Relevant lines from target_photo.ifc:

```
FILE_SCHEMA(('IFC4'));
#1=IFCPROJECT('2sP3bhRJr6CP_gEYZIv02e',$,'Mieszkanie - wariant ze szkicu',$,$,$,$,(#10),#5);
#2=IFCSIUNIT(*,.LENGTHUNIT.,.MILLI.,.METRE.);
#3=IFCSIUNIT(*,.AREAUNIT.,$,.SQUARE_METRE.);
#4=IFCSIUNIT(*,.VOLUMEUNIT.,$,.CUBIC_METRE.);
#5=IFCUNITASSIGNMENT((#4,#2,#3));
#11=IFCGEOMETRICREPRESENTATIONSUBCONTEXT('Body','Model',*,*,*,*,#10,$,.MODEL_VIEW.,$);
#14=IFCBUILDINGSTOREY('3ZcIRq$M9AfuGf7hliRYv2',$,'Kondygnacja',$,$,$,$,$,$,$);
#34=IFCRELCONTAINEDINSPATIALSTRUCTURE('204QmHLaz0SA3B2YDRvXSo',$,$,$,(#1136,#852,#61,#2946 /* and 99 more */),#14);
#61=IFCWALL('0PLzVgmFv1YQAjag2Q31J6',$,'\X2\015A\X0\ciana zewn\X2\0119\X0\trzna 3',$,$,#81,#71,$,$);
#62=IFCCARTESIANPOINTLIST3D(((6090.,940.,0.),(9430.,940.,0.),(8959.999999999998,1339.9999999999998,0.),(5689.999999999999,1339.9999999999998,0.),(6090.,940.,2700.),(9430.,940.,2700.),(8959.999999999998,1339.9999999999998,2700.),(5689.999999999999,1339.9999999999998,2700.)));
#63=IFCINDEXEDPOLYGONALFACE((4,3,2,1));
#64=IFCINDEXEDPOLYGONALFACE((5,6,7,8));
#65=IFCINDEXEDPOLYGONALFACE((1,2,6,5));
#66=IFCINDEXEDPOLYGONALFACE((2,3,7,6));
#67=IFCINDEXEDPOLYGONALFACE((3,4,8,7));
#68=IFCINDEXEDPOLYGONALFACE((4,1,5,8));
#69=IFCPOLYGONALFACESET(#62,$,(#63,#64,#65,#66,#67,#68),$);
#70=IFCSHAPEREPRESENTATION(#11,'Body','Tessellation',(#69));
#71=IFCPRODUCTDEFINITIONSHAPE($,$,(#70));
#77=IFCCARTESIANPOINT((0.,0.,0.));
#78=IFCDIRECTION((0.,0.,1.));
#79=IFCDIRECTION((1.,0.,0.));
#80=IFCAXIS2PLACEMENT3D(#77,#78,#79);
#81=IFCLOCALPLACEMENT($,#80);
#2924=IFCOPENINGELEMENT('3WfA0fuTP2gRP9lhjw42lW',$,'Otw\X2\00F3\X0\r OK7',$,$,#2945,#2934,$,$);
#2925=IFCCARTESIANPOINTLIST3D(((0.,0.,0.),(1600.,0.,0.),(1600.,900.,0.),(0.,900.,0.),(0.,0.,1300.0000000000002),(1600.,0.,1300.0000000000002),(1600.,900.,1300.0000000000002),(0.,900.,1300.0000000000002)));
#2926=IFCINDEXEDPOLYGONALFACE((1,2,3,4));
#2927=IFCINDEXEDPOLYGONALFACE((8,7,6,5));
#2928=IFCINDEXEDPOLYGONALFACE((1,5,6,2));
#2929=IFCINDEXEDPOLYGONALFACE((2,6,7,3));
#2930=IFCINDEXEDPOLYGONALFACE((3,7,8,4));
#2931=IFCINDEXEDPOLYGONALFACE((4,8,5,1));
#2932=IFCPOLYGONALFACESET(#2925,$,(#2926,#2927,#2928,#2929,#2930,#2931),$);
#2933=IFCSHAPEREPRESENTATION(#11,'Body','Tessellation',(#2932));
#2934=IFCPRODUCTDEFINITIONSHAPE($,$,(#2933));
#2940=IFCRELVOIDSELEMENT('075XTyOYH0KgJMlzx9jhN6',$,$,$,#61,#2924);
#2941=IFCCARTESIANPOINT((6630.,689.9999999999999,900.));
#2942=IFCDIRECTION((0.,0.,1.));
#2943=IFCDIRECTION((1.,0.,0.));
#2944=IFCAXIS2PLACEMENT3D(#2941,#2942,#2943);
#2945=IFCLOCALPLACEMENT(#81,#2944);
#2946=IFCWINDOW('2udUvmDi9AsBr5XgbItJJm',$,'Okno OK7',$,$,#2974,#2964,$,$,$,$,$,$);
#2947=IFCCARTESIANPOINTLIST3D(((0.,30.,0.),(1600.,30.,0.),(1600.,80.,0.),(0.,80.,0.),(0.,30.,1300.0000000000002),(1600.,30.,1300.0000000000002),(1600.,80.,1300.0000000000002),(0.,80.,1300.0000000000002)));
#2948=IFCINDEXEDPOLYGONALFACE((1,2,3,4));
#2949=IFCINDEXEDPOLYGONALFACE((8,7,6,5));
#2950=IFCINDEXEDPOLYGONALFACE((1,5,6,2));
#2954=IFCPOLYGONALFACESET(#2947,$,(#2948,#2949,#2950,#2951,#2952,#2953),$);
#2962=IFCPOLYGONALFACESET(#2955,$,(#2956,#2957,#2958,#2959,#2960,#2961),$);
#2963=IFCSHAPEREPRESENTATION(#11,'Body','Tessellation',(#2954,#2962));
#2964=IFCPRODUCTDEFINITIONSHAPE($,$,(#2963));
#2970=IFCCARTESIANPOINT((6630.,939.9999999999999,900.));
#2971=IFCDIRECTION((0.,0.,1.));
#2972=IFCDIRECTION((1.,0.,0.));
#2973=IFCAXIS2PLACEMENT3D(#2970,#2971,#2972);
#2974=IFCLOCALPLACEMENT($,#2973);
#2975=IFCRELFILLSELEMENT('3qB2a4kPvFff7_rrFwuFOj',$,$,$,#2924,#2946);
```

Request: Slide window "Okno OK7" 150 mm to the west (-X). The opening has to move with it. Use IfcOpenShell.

```python
import ifcopenshell
import ifcopenshell.api.geometry
import ifcopenshell.util.placement

model = ifcopenshell.open("target_photo.ifc")

window = model.by_guid("2udUvmDi9AsBr5XgbItJJm")
opening = window.FillsVoids[0].RelatingOpeningElement
wall = opening.VoidsElements[0].RelatingBuildingElement

wall_matrix = ifcopenshell.util.placement.get_local_placement(wall.ObjectPlacement)
shift = wall_matrix[:3, 0] * -150.0
before = ifcopenshell.util.placement.get_local_placement(window.ObjectPlacement)[:3, 3].copy()

# The window is not placed relative to its opening, so move both.
for product in (opening, window):
    matrix = ifcopenshell.util.placement.get_local_placement(product.ObjectPlacement)
    matrix[:3, 3] += shift
    ifcopenshell.api.geometry.edit_object_placement(model, product=product, matrix=matrix, is_si=False)

after = ifcopenshell.util.placement.get_local_placement(window.ObjectPlacement)[:3, 3]
print("window moved by", (after - before).round(3) + 0.0)

model.write("target_photo_v2.ifc")
```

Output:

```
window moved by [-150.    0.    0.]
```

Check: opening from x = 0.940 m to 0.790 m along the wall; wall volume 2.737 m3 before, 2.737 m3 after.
